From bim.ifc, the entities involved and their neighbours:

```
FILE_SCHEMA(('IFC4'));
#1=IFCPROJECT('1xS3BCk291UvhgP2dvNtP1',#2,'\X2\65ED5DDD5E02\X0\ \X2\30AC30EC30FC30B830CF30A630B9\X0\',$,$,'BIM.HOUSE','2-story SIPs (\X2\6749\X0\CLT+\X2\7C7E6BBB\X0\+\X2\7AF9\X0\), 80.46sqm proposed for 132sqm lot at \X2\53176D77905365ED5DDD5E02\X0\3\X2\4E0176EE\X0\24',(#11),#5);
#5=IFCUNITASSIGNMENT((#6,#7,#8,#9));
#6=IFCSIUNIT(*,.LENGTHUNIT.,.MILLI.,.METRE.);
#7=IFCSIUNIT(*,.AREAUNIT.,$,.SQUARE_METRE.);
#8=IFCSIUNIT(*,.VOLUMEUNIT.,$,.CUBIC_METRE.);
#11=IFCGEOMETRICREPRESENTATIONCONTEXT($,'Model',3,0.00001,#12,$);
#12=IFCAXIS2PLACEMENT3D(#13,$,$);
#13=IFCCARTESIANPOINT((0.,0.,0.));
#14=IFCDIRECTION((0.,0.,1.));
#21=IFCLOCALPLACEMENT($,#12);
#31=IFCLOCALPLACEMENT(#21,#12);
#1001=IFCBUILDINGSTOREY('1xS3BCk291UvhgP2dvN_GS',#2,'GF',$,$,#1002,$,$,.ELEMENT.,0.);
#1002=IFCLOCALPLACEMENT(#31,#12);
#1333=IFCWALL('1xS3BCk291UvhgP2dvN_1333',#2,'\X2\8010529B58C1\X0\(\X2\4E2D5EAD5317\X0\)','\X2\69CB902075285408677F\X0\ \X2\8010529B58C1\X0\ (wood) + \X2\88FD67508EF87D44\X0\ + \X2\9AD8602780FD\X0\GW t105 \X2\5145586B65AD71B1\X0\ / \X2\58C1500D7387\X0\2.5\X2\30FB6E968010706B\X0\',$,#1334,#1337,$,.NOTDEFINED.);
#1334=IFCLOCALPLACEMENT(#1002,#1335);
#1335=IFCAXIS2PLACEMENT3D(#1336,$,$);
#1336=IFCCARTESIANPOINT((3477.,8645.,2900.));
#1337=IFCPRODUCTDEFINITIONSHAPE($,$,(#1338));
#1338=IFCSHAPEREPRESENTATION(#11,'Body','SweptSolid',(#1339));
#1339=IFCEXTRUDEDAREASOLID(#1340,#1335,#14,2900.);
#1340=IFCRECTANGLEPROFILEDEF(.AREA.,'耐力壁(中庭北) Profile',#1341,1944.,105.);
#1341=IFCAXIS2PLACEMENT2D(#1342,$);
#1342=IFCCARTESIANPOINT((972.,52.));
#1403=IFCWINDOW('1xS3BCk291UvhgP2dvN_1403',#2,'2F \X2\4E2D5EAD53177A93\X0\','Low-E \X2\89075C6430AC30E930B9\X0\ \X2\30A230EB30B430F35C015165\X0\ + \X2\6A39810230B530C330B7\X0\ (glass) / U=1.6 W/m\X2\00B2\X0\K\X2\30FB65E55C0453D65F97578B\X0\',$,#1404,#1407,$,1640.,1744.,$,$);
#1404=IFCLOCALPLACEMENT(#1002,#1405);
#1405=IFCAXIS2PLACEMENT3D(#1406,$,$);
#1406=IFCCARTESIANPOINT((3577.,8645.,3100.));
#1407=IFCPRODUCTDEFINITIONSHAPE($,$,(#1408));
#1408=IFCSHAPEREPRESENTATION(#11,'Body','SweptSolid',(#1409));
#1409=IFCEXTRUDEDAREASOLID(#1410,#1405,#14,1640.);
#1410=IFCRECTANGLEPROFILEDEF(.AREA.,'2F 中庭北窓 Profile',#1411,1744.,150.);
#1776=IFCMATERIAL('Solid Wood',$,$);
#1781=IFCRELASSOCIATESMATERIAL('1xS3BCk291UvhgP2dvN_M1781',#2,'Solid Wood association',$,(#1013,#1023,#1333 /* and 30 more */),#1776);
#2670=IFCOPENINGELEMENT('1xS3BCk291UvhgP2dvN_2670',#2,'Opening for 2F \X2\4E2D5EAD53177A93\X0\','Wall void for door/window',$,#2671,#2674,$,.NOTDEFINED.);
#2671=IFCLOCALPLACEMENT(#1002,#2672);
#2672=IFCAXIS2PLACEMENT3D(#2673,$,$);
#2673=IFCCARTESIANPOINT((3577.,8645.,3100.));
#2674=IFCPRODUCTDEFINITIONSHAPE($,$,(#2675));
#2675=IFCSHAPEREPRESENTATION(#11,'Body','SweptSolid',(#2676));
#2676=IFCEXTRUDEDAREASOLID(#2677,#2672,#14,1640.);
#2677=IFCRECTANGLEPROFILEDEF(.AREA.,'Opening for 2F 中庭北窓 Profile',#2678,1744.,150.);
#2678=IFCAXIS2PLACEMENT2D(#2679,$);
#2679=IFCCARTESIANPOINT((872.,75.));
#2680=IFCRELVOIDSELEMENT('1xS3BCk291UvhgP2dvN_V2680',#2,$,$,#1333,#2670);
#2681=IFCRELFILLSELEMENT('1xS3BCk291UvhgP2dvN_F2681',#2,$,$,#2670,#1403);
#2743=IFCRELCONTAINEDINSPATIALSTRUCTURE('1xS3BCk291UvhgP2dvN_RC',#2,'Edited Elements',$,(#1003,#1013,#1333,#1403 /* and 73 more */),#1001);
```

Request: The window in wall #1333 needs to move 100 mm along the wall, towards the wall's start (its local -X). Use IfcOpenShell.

```python
import ifcopenshell
import ifcopenshell.api.geometry
import ifcopenshell.util.placement
import ifcopenshell.util.unit

model = ifcopenshell.open("bim.ifc")
unit_scale = ifcopenshell.util.unit.calculate_unit_scale(model)

window = model.by_id(1403)
opening = window.FillsVoids[0].RelatingOpeningElement
wall = opening.VoidsElements[0].RelatingBuildingElement

wall_matrix = ifcopenshell.util.placement.get_local_placement(wall.ObjectPlacement)
shift = wall_matrix[:3, 0] * -0.1 / unit_scale
before = ifcopenshell.util.placement.get_local_placement(window.ObjectPlacement)[:3, 3].copy()

# The window is not placed relative to its opening, so move both.
for product in (opening, window):
    matrix = ifcopenshell.util.placement.get_local_placement(product.ObjectPlacement)
    matrix[:3, 3] += shift
    ifcopenshell.api.geometry.edit_object_placement(model, product=product, matrix=matrix, is_si=False)

after = ifcopenshell.util.placement.get_local_placement(window.ObjectPlacement)[:3, 3]
print("window moved by", (after - before).round(3) + 0.0)

model.write("bim_v2.ifc")
```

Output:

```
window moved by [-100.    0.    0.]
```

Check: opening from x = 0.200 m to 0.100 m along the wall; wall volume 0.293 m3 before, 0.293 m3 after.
